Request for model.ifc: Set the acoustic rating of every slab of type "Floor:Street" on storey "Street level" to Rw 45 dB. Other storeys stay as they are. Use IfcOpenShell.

First a look at what the model holds.

```python
import ifcopenshell
import ifcopenshell.util.element

model = ifcopenshell.open("model.ifc")
print(model.schema)
storey = next(s for s in model.by_type("IfcBuildingStorey") if s.Name == "Street level")
slabs = [e for e in ifcopenshell.util.element.get_decomposition(storey) if e.is_a("IfcSlab")]
seen = {}
for e in slabs:
    element_type = ifcopenshell.util.element.get_type(e)
    key = (element_type.Name if element_type != e and element_type else None, ifcopenshell.util.element.get_pset(e, "Pset_SlabCommon", "AcousticRating"))
    seen[key] = seen.get(key, 0) + 1
for (name, value), count in sorted(seen.items(), key=str):
    print(count, "x", name, "|", value)
```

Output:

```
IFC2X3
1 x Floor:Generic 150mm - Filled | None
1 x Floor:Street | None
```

```python
import ifcopenshell
import ifcopenshell.api.pset
import ifcopenshell.util.element

model = ifcopenshell.open("model.ifc")

storey = next(s for s in model.by_type("IfcBuildingStorey") if s.Name == "Street level")
slabs = [e for e in ifcopenshell.util.element.get_decomposition(storey) if e.is_a("IfcSlab")]

count = 0
for e in slabs:
    element_type = ifcopenshell.util.element.get_type(e)
    if element_type in (None, e) or element_type.Name != "Floor:Street":
        continue
    # add_pset returns the element's existing set when there is one.
    pset = ifcopenshell.api.pset.add_pset(model, product=e, name="Pset_SlabCommon")
    ifcopenshell.api.pset.edit_pset(model, pset=pset, properties={"AcousticRating": "Rw 45 dB"})
    count += 1

print(count, "slabs updated")

model.write("model_rev.ifc")
```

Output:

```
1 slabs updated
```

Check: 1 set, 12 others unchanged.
